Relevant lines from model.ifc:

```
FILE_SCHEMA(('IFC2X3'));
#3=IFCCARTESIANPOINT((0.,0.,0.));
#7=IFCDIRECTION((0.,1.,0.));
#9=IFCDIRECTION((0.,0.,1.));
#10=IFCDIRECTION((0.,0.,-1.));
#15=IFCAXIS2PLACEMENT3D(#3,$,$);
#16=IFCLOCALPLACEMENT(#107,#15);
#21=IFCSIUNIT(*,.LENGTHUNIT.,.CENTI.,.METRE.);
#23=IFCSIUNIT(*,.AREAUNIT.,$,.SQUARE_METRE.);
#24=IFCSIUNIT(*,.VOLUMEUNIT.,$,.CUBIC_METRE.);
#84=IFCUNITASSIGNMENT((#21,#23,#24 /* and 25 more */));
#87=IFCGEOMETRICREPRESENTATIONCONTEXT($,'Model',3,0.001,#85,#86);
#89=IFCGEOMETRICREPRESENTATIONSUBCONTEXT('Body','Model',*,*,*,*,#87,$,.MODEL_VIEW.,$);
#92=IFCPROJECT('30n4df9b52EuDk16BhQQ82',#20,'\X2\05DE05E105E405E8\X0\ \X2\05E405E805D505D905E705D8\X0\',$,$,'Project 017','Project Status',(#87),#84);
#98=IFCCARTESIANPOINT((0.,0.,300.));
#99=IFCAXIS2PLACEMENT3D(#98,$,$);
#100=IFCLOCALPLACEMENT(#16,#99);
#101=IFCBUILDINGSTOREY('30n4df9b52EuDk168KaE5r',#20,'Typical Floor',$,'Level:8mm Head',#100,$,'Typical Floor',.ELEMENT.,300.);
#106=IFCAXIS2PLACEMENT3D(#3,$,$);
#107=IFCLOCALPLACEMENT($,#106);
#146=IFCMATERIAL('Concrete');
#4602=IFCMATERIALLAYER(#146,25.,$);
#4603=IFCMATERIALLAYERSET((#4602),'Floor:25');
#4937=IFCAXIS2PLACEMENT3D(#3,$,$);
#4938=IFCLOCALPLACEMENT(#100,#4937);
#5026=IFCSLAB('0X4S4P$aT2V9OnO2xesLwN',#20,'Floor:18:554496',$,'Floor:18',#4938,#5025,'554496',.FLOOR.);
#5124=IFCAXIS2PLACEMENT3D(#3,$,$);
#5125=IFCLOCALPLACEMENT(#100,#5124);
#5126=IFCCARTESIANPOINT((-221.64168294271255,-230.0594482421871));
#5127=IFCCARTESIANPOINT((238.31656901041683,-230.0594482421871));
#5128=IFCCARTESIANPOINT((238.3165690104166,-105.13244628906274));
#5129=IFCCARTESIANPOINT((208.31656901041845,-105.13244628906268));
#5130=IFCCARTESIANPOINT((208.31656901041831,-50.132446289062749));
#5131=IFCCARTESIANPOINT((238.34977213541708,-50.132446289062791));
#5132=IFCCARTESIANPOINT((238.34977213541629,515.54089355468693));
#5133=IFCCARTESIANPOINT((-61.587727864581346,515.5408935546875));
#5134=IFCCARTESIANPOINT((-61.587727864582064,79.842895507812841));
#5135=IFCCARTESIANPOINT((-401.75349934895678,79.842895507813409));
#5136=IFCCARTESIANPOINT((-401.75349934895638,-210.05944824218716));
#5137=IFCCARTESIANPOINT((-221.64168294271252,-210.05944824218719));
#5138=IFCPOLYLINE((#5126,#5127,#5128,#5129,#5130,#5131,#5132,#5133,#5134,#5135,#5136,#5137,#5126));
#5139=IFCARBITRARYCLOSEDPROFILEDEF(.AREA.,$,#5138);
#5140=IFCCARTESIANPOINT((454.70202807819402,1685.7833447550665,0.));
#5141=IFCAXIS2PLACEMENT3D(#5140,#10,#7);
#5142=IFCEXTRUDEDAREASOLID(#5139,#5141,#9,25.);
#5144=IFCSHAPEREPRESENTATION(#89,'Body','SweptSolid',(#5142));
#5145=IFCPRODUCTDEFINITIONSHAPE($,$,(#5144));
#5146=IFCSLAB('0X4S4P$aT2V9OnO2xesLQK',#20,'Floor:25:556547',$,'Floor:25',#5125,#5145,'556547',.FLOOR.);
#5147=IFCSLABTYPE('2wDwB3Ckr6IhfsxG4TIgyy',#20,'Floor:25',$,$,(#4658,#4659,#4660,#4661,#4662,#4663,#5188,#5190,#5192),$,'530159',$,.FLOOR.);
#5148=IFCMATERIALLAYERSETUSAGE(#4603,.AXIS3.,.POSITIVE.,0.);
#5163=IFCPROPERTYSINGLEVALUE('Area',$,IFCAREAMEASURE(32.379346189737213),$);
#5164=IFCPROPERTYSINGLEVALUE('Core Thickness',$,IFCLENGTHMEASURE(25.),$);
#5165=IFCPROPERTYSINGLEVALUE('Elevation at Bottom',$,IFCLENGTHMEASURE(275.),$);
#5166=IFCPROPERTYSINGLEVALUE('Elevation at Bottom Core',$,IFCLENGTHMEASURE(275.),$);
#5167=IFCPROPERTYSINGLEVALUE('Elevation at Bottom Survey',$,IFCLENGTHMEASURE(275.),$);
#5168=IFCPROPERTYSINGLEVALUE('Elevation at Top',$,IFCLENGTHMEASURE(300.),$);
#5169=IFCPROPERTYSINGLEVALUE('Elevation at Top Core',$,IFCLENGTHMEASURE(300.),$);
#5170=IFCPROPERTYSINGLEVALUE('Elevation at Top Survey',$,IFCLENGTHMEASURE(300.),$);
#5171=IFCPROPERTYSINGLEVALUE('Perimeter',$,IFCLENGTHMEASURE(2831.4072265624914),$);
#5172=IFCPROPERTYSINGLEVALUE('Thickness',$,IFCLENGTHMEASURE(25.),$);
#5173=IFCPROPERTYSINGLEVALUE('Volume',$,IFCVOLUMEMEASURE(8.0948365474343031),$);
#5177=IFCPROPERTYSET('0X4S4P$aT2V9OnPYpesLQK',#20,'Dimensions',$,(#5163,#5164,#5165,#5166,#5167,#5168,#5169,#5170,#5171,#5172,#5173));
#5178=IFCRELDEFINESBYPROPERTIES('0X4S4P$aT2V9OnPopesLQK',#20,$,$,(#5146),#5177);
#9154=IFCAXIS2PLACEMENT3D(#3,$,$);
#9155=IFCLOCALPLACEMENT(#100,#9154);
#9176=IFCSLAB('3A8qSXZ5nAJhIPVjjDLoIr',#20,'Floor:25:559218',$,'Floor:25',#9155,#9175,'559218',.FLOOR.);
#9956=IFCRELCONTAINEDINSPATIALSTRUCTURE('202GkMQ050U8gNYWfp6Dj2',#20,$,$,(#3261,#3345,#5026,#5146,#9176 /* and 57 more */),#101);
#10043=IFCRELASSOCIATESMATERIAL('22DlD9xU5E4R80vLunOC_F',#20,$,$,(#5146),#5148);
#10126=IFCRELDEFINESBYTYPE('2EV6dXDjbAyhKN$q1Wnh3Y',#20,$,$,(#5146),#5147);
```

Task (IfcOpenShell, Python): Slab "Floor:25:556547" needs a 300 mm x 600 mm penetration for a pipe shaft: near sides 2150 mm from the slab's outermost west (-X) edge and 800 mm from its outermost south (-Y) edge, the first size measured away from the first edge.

```python
import numpy as np
import ifcopenshell
import ifcopenshell.api.feature
import ifcopenshell.api.geometry
import ifcopenshell.api.pset
import ifcopenshell.api.root
import ifcopenshell.geom
import ifcopenshell.util.element
import ifcopenshell.util.placement
import ifcopenshell.util.representation
import ifcopenshell.util.shape
import ifcopenshell.util.unit

model = ifcopenshell.open("model.ifc")
unit_scale = ifcopenshell.util.unit.calculate_unit_scale(model)
area_scale = ifcopenshell.util.unit.calculate_unit_scale(model, "AREAUNIT")
volume_scale = ifcopenshell.util.unit.calculate_unit_scale(model, "VOLUMEUNIT")
settings = ifcopenshell.geom.settings()


def volume(element):
    """Net volume in cubic metres, openings subtracted."""
    shape = ifcopenshell.geom.create_shape(settings, element)
    return ifcopenshell.util.shape.get_volume(shape.geometry)


slab = model.by_id(5146)
before = volume(slab)

# Extent in the slab's own axes, in metres. The edges named are its -X and -Y sides.
slab_shape = ifcopenshell.geom.create_shape(settings, slab)
vertices = ifcopenshell.util.shape.get_vertices(slab_shape.geometry)
x_min, y_min, bottom = vertices.min(axis=0)
top = vertices[:, 2].max()

opening = ifcopenshell.api.root.create_entity(model, ifc_class="IfcOpeningElement", name="Pipe shaft opening")
context = ifcopenshell.util.representation.get_context(model, "Model", "Body", "MODEL_VIEW")
width, depth = 0.3, 0.6
outline = [(0.0, 0.0), (width, 0.0), (width, depth), (0.0, depth), (0.0, 0.0)]
# Overshoot both faces by 50 mm so the cut is clean.
shape = ifcopenshell.api.geometry.add_slab_representation(
    model, context=context, depth=top - bottom + 0.1, polyline=outline
)
ifcopenshell.api.geometry.assign_representation(model, product=opening, representation=shape)

matrix = ifcopenshell.util.placement.get_local_placement(slab.ObjectPlacement)
matrix[:, 3] = matrix @ np.append(np.array([x_min + 2.15, y_min + 0.8, bottom - 0.05]) / unit_scale, 1.0)
ifcopenshell.api.geometry.edit_object_placement(model, product=opening, matrix=matrix, is_si=False)
ifcopenshell.api.feature.add_feature(model, feature=opening, element=slab)

after = volume(slab)

# Update the slab's stored quantities.
pset = model.by_id(ifcopenshell.util.element.get_pset(slab, "Dimensions", should_inherit=False)["id"])
ifcopenshell.api.pset.edit_pset(model, pset=pset, properties={
    "Area": model.create_entity("IfcAreaMeasure", after / (top - bottom) / area_scale),
    "Volume": model.create_entity("IfcVolumeMeasure", after / volume_scale),
})

print(f"slab volume {before:.3f} -> {after:.3f} m3")

model.write("model_v2.ifc")
```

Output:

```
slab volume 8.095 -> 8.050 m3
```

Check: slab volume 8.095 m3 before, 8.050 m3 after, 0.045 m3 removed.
